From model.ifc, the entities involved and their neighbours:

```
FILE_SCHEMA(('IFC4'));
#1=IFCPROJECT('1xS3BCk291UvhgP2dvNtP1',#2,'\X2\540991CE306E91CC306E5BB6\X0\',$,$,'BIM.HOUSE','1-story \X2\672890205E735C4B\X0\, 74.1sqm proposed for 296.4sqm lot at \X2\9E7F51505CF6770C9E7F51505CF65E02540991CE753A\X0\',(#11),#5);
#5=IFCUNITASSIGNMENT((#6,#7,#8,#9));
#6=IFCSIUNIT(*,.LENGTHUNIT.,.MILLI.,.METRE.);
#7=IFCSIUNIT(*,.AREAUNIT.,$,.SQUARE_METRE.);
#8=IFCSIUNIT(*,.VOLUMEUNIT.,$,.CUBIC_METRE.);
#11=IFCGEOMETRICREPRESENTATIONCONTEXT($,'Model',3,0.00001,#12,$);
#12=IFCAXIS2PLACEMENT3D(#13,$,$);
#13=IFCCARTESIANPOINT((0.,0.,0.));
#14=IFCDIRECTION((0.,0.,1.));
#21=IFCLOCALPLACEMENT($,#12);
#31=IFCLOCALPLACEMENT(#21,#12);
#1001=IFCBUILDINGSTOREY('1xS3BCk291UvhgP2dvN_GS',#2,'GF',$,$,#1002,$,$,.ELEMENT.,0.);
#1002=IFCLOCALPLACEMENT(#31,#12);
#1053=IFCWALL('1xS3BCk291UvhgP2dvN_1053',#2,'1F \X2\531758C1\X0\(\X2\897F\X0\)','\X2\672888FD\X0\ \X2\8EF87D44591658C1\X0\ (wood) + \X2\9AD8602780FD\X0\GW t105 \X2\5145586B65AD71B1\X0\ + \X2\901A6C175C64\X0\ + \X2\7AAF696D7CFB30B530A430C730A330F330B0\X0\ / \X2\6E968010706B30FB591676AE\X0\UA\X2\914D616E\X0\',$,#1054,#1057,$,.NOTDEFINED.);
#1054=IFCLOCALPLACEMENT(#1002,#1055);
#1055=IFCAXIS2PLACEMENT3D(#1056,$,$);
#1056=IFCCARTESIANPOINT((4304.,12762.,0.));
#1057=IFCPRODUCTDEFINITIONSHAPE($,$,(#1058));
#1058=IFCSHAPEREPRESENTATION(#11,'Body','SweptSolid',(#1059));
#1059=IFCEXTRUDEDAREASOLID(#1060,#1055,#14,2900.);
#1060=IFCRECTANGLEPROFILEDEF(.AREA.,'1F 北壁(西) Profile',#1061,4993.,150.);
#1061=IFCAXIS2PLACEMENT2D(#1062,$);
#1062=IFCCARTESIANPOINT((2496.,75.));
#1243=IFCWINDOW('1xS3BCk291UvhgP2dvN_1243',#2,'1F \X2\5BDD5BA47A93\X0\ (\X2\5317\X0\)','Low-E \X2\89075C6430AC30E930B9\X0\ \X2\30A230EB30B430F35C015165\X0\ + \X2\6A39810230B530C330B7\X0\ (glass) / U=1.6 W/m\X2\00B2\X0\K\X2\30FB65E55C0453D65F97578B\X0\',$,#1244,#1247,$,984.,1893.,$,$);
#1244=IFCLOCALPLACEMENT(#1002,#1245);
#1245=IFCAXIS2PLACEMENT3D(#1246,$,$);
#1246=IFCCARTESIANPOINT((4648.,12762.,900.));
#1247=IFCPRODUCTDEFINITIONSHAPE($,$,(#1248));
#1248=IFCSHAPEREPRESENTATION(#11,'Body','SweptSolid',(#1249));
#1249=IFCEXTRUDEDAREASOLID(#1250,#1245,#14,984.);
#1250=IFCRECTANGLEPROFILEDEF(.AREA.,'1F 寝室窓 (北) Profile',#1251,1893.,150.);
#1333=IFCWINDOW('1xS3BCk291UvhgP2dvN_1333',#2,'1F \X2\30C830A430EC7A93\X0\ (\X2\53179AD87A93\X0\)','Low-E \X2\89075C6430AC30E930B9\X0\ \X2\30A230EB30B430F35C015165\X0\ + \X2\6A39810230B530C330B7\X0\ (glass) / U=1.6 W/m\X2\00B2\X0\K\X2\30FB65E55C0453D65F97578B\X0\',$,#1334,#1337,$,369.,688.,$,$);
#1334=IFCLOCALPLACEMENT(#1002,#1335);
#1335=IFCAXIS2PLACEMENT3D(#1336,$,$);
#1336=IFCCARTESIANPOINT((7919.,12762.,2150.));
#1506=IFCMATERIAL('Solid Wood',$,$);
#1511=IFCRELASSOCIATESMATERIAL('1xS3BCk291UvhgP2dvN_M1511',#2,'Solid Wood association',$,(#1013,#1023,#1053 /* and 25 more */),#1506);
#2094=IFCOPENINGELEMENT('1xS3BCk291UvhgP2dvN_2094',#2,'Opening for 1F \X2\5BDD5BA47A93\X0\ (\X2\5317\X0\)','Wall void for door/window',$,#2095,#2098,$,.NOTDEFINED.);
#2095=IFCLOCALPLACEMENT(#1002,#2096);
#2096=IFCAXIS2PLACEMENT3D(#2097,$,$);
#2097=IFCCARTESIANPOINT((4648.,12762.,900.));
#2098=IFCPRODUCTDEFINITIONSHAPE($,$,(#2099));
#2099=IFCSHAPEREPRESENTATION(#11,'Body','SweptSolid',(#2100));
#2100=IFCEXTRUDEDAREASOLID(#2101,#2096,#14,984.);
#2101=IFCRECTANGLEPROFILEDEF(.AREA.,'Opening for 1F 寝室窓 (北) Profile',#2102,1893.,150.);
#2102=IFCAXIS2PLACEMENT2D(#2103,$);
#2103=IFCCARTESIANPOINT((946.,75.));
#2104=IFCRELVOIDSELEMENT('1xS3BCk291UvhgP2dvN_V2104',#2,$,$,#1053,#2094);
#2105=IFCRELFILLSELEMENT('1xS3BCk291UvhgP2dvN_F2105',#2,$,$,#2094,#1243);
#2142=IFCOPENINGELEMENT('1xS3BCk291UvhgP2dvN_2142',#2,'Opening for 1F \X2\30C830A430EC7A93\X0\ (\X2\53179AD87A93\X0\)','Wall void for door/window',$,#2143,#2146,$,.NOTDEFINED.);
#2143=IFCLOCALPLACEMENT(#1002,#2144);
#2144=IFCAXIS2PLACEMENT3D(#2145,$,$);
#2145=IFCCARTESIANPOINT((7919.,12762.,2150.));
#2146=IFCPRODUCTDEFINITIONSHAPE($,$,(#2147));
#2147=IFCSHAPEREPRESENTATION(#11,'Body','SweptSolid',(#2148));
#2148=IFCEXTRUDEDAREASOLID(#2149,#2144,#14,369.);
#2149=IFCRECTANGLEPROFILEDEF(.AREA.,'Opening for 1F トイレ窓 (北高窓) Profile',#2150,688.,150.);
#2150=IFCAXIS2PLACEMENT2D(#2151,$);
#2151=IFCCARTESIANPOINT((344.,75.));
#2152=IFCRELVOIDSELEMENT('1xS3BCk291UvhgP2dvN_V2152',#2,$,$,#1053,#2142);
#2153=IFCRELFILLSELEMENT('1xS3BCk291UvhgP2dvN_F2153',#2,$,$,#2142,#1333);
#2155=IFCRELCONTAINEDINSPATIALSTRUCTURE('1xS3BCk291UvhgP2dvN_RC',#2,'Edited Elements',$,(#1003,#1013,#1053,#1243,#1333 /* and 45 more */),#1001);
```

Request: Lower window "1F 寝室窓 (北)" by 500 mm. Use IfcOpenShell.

```python
import numpy as np
import ifcopenshell
import ifcopenshell.api.geometry
import ifcopenshell.util.placement
import ifcopenshell.util.unit

model = ifcopenshell.open("model.ifc")
unit_scale = ifcopenshell.util.unit.calculate_unit_scale(model)

window = model.by_guid("1xS3BCk291UvhgP2dvN_1243")
opening = window.FillsVoids[0].RelatingOpeningElement
dz = -0.5 / unit_scale

shift = np.array([0.0, 0.0, dz])
# The window is not placed relative to its opening, so move both.
for product in (opening, window):
    matrix = ifcopenshell.util.placement.get_local_placement(product.ObjectPlacement)
    matrix[:3, 3] += shift
    ifcopenshell.api.geometry.edit_object_placement(model, product=product, matrix=matrix, is_si=False)

print(f"moved by {dz * unit_scale:+.3f} m")

model.write("model-out.ifc")
```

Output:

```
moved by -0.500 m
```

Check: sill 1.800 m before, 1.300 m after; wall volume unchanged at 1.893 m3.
